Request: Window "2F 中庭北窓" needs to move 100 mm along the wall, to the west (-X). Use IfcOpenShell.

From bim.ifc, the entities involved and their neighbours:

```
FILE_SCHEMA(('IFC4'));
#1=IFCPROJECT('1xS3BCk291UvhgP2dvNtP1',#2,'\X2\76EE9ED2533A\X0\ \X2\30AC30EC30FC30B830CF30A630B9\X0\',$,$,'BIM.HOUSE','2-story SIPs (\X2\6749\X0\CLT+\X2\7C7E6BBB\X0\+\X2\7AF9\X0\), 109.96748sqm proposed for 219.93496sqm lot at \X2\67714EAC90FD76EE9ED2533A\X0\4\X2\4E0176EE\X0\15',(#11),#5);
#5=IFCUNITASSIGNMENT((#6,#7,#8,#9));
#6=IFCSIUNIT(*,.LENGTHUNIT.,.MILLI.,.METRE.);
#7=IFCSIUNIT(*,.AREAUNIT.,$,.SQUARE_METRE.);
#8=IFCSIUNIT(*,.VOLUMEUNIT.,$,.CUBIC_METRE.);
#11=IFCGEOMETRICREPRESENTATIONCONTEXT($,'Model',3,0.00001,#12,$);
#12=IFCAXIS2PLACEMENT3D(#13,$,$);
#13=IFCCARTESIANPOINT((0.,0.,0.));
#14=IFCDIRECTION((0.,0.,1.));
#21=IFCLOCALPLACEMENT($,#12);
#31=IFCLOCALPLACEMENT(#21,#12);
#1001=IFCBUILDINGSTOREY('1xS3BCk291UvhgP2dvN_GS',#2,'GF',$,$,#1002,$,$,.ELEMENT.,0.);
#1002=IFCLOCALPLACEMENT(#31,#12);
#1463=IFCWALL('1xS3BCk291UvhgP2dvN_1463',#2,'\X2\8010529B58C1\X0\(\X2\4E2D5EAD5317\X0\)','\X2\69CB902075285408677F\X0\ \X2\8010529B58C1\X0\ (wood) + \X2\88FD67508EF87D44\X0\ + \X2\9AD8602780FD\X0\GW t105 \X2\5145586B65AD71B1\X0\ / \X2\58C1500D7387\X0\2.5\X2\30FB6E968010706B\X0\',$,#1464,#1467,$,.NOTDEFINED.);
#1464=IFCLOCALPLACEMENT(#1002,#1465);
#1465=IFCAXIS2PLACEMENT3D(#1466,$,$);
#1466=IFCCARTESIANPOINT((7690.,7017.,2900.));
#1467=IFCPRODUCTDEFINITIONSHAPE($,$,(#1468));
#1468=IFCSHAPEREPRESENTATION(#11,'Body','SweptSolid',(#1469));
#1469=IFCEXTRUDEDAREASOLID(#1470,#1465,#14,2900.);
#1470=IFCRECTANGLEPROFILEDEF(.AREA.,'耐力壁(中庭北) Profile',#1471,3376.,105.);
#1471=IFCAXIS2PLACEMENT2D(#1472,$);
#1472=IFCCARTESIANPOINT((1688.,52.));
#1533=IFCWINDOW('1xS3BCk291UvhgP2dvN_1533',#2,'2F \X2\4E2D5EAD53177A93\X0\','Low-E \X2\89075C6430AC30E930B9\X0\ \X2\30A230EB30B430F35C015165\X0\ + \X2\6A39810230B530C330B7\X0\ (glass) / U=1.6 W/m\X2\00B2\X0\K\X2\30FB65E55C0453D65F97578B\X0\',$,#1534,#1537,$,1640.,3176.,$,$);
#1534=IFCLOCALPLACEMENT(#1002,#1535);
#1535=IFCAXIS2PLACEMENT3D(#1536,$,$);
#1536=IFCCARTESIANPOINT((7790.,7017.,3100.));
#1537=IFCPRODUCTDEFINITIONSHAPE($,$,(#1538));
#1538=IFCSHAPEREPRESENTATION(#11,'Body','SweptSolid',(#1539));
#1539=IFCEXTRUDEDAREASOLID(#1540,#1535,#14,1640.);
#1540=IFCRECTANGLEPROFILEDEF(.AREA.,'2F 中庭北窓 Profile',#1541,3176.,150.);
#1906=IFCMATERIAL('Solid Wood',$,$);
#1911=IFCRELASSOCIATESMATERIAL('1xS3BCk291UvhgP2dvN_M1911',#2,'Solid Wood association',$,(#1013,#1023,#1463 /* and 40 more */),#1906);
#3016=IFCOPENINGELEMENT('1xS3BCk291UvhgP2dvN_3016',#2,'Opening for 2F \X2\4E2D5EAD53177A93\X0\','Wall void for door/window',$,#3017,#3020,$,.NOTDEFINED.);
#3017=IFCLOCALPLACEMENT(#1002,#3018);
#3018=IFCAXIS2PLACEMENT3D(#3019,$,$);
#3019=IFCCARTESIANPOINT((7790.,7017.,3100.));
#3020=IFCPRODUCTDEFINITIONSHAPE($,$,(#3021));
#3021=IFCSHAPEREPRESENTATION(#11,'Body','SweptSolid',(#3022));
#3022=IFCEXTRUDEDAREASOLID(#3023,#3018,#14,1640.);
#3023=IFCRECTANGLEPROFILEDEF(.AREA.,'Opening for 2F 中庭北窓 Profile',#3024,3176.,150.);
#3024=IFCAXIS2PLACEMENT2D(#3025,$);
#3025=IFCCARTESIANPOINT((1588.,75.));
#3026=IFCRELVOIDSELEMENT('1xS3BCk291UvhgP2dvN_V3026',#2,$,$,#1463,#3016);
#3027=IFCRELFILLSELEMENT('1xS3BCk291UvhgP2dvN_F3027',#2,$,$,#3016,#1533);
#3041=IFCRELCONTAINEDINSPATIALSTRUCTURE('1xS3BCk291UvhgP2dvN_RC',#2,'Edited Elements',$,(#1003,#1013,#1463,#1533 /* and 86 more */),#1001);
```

```python
import ifcopenshell
import ifcopenshell.api.geometry
import ifcopenshell.util.placement
import ifcopenshell.util.unit

model = ifcopenshell.open("bim.ifc")
unit_scale = ifcopenshell.util.unit.calculate_unit_scale(model)

window = model.by_id(1533)
opening = window.FillsVoids[0].RelatingOpeningElement
wall = opening.VoidsElements[0].RelatingBuildingElement

wall_matrix = ifcopenshell.util.placement.get_local_placement(wall.ObjectPlacement)
shift = wall_matrix[:3, 0] * -0.1 / unit_scale
before = ifcopenshell.util.placement.get_local_placement(window.ObjectPlacement)[:3, 3].copy()

# The window is not placed relative to its opening, so move both.
for product in (opening, window):
    matrix = ifcopenshell.util.placement.get_local_placement(product.ObjectPlacement)
    matrix[:3, 3] += shift
    ifcopenshell.api.geometry.edit_object_placement(model, product=product, matrix=matrix, is_si=False)

after = ifcopenshell.util.placement.get_local_placement(window.ObjectPlacement)[:3, 3]
print("window moved by", (after - before).round(3) + 0.0)

model.write("bim_v2.ifc")
```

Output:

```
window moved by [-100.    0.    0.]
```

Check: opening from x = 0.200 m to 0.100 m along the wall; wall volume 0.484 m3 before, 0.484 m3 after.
